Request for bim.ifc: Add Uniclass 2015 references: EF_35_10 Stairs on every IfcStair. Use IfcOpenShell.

First a look at what the model holds.

```python
import ifcopenshell

model = ifcopenshell.open("bim.ifc")
print(model.schema)
print("classifications:", [c.Name for c in model.by_type("IfcClassification")])
for ifc_class in ("IfcDoor", "IfcRoof", "IfcStair", "IfcWall", "IfcWindow"):
    print(ifc_class, len(model.by_type(ifc_class)))
```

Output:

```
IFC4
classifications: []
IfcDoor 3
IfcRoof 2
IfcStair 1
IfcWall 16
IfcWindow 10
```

```python
import ifcopenshell
import ifcopenshell.api.classification

model = ifcopenshell.open("bim.ifc")

system = ifcopenshell.api.classification.add_classification(model, classification="Uniclass 2015")

codes = {
    "IfcStair": ("EF_35_10", "Stairs"),
}
for ifc_class, (code, name) in codes.items():
    products = model.by_type(ifc_class)
    ifcopenshell.api.classification.add_reference(
        model, products=products, classification=system, identification=code, name=name
    )
    print(code, len(products))

model.write("bim_v2.ifc")
```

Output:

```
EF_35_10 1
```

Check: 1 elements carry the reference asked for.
